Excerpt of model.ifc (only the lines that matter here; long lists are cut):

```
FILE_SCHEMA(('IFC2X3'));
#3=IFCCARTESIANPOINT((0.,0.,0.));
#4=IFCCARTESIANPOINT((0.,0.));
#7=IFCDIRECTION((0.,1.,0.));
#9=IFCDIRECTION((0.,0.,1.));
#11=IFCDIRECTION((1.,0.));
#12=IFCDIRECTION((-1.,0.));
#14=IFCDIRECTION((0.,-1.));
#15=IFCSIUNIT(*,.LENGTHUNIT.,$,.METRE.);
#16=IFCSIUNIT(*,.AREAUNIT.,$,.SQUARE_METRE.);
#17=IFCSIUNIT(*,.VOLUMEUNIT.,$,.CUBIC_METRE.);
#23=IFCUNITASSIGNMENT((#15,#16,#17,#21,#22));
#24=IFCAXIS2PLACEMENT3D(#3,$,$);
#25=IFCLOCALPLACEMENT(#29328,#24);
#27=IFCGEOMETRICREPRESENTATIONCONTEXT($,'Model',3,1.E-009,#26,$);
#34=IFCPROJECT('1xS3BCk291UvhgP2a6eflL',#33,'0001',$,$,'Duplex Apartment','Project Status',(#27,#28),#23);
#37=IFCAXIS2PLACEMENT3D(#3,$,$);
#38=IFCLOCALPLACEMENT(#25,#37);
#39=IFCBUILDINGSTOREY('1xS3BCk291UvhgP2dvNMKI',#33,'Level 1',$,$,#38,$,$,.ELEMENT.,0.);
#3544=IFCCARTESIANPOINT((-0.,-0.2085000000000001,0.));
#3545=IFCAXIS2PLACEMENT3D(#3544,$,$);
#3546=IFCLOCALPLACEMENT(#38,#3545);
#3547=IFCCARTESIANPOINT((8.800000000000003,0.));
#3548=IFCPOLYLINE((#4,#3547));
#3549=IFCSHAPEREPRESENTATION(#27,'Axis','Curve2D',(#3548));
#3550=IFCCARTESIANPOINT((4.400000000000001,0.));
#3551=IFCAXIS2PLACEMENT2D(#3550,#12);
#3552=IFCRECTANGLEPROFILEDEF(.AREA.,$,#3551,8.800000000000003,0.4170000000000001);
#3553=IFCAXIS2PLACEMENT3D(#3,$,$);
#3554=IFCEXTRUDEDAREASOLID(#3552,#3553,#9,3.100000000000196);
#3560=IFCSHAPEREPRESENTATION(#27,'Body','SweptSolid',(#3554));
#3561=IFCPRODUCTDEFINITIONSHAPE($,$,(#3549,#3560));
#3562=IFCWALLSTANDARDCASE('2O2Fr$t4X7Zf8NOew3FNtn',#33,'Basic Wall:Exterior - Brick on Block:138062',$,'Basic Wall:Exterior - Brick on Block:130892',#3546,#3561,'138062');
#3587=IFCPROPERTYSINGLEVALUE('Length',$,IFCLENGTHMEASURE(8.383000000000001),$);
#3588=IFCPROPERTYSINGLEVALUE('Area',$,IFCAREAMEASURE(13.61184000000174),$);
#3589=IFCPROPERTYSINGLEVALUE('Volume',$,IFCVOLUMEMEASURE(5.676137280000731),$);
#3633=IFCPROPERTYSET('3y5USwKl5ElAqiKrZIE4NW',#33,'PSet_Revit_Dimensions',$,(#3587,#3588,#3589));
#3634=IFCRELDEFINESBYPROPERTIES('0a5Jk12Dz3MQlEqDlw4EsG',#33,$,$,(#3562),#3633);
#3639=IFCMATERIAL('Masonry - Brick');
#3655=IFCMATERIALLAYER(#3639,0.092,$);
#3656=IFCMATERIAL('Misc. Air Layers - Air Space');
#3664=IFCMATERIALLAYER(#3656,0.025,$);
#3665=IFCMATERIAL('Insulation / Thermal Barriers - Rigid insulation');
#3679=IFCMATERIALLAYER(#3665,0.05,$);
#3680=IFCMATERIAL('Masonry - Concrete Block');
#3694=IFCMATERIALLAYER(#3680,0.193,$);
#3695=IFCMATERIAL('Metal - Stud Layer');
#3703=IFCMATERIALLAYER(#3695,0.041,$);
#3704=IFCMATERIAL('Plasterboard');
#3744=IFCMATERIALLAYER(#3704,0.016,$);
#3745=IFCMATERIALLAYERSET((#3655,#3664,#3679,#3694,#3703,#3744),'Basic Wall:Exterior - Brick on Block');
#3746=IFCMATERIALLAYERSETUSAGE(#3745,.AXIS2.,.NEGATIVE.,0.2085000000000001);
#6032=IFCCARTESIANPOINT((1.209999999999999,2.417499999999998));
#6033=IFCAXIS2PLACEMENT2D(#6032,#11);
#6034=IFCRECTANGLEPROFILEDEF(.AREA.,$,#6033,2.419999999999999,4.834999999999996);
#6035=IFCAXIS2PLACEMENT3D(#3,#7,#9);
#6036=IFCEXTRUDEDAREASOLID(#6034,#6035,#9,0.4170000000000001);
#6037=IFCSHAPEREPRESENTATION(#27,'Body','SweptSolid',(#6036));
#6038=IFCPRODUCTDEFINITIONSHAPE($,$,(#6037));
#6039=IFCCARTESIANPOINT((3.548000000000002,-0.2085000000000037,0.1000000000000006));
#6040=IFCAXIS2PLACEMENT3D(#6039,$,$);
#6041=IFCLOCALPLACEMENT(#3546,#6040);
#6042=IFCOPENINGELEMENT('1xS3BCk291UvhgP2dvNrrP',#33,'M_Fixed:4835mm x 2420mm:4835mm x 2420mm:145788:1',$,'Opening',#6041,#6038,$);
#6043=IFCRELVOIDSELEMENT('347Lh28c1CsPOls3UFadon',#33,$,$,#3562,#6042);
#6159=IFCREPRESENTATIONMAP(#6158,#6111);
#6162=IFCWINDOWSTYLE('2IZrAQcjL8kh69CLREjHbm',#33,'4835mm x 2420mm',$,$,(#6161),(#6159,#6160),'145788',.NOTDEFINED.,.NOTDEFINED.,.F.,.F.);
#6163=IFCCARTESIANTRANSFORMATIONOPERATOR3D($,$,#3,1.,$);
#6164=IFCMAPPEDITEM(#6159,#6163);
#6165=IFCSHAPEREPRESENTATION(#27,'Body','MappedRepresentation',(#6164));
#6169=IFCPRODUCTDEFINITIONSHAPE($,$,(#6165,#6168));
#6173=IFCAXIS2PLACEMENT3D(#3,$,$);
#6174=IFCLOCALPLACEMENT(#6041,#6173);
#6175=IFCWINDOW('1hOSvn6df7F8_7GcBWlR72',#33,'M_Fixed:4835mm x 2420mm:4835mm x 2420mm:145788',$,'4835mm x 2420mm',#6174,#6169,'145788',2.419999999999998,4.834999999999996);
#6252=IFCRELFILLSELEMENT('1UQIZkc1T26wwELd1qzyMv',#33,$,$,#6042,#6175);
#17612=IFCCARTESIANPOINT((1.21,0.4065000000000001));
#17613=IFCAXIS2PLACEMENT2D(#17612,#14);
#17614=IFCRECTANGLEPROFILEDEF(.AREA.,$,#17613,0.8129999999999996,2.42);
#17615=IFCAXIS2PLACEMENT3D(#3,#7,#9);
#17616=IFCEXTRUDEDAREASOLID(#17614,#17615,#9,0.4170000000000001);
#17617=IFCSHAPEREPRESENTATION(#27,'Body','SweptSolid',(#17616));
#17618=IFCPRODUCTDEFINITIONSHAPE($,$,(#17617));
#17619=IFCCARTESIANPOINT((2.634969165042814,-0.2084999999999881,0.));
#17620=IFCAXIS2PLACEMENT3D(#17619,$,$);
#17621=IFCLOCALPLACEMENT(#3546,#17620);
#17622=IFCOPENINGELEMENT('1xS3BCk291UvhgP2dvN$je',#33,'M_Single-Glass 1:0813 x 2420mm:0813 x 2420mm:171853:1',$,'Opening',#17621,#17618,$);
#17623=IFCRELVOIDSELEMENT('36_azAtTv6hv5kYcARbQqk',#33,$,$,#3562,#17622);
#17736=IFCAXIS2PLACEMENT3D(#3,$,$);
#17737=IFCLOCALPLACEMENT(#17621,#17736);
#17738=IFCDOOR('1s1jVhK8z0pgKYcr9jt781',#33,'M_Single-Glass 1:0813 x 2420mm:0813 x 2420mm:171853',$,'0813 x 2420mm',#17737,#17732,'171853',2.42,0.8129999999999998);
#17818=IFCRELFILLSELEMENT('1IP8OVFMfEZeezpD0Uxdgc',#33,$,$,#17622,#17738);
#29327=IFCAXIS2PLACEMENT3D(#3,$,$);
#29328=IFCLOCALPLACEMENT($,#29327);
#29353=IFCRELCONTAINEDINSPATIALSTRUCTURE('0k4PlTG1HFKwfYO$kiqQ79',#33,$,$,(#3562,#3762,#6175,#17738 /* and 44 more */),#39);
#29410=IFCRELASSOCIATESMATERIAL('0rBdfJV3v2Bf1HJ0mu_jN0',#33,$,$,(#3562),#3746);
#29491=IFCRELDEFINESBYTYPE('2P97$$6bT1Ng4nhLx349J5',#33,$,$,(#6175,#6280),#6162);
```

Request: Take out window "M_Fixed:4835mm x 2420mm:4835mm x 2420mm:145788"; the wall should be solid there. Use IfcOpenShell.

```python
import ifcopenshell
import ifcopenshell.api.feature
import ifcopenshell.api.pset
import ifcopenshell.api.root
import ifcopenshell.geom
import ifcopenshell.util.element
import ifcopenshell.util.shape
import ifcopenshell.util.unit

model = ifcopenshell.open("model.ifc")
area_scale = ifcopenshell.util.unit.calculate_unit_scale(model, "AREAUNIT")
volume_scale = ifcopenshell.util.unit.calculate_unit_scale(model, "VOLUMEUNIT")
settings = ifcopenshell.geom.settings()


def volume(element):
    """Net volume in cubic metres, openings subtracted."""
    shape = ifcopenshell.geom.create_shape(settings, element)
    return ifcopenshell.util.shape.get_volume(shape.geometry)


window = model.by_guid("1hOSvn6df7F8_7GcBWlR72")
opening = window.FillsVoids[0].RelatingOpeningElement
wall = opening.VoidsElements[0].RelatingBuildingElement
before = volume(wall)

ifcopenshell.api.root.remove_product(model, product=window)
ifcopenshell.api.feature.remove_feature(model, feature=opening)

after = volume(wall)
thickness = 0.417  # wall thickness in metres

# Update the wall's stored quantities.
pset = model.by_id(ifcopenshell.util.element.get_pset(wall, "PSet_Revit_Dimensions", should_inherit=False)["id"])
ifcopenshell.api.pset.edit_pset(model, pset=pset, properties={
    "Area": model.create_entity("IfcAreaMeasure", after / thickness / area_scale),
    "Volume": model.create_entity("IfcVolumeMeasure", after / volume_scale),
})

print(f"wall volume {before:.3f} -> {after:.3f} m3")

model.write("model_edited.ifc")
```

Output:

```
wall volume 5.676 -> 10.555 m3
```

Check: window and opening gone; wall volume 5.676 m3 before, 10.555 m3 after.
